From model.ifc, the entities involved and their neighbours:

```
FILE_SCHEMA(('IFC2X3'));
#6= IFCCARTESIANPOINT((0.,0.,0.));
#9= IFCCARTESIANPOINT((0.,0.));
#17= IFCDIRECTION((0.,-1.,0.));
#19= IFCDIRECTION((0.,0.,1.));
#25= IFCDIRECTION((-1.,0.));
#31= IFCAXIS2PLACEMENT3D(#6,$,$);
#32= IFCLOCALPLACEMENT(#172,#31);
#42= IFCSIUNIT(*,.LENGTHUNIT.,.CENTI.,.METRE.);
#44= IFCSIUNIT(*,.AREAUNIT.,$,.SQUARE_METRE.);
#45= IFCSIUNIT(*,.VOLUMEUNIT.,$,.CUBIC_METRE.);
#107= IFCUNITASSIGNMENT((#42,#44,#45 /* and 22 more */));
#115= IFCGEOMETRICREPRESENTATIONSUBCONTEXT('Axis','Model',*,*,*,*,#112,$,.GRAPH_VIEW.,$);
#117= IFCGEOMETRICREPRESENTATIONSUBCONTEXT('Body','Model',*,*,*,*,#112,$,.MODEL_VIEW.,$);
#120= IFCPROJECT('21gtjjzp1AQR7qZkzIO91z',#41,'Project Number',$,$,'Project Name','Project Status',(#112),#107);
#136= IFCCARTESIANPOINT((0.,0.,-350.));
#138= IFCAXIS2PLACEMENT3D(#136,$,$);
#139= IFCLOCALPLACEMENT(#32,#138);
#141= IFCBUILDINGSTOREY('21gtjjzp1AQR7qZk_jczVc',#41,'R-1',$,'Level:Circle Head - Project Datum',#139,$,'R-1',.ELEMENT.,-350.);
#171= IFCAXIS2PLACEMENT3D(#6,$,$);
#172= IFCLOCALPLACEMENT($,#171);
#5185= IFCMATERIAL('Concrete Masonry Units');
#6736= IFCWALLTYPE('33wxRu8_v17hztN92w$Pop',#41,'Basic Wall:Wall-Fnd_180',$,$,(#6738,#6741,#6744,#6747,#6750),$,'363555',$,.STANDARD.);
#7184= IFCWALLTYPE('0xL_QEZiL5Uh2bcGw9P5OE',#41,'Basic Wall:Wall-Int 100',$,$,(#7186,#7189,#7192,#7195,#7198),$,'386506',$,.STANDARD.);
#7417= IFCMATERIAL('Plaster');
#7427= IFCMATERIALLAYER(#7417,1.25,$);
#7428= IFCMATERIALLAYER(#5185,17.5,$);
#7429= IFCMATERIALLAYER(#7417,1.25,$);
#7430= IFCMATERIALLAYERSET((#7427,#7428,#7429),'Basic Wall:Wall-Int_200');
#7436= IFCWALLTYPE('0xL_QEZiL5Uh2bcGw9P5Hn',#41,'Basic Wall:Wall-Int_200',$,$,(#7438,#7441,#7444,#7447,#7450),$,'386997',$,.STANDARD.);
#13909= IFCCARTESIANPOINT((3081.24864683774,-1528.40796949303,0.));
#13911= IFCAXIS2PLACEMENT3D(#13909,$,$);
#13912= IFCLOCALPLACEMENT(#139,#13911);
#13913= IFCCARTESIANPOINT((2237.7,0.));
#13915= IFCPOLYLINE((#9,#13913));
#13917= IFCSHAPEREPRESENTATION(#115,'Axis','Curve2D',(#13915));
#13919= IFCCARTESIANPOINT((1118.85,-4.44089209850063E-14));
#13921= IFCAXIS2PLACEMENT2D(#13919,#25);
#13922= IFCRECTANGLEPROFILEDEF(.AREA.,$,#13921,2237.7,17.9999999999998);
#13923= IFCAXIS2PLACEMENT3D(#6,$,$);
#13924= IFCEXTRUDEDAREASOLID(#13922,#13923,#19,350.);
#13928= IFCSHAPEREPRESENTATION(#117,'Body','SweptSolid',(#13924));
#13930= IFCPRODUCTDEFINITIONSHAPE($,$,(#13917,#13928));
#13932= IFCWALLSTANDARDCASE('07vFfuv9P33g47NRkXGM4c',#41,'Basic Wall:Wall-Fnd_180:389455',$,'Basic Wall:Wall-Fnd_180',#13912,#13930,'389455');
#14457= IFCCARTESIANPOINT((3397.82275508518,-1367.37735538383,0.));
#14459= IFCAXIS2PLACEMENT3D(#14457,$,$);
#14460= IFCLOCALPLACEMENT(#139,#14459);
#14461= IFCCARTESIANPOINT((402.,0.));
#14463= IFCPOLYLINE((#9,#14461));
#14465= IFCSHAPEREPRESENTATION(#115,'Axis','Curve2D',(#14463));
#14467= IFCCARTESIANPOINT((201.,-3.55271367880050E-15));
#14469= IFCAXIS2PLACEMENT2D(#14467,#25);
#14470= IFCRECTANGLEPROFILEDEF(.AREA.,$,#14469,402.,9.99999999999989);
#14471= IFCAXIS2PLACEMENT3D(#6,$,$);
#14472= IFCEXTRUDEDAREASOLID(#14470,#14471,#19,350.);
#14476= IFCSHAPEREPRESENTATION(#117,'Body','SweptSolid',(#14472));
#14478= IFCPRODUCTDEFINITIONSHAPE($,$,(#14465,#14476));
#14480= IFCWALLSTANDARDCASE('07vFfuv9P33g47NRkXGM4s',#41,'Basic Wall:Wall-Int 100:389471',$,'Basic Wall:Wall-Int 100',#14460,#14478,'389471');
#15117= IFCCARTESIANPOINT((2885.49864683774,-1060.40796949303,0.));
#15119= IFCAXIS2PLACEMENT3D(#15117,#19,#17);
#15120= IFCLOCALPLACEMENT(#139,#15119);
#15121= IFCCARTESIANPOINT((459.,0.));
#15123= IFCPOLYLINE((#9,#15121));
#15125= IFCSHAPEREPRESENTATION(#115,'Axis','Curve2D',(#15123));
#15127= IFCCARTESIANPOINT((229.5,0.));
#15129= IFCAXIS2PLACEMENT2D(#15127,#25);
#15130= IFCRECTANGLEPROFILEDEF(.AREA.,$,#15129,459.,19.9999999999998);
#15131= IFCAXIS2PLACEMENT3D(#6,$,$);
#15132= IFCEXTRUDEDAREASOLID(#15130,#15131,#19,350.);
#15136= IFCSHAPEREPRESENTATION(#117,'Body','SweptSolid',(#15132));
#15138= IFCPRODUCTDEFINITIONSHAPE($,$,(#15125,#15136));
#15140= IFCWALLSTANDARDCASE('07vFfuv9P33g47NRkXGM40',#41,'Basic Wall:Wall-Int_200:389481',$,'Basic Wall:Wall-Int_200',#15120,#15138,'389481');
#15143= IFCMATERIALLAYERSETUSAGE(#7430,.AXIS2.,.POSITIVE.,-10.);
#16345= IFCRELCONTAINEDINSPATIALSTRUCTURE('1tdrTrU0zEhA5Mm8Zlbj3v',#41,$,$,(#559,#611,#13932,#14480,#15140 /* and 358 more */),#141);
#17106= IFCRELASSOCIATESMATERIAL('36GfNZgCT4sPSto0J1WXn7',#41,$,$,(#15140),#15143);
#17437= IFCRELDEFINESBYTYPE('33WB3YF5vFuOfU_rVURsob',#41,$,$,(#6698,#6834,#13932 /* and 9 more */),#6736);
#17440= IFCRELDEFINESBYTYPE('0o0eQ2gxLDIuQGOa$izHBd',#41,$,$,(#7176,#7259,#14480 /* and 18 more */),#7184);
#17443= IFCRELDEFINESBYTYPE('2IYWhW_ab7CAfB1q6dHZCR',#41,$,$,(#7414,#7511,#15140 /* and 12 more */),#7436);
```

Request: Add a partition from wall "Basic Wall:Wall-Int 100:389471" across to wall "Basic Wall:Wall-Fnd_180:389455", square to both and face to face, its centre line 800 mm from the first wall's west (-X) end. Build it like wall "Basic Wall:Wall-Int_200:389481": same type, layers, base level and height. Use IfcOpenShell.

```python
import numpy as np
import ifcopenshell
import ifcopenshell.api.geometry
import ifcopenshell.api.material
import ifcopenshell.api.pset
import ifcopenshell.api.root
import ifcopenshell.api.spatial
import ifcopenshell.api.type
import ifcopenshell.geom
import ifcopenshell.util.element
import ifcopenshell.util.placement
import ifcopenshell.util.representation
import ifcopenshell.util.shape
import ifcopenshell.util.unit

model = ifcopenshell.open("model.ifc")
unit_scale = ifcopenshell.util.unit.calculate_unit_scale(model)
settings = ifcopenshell.geom.settings()
settings.set("use-world-coords", True)

start_wall = model.by_id(14480)
end_wall = model.by_guid("07vFfuv9P33g47NRkXGM4c")
like = model.by_id(15140)
matrix = ifcopenshell.util.placement.get_local_placement(start_wall.ObjectPlacement)
matrix[:3, 3] *= unit_scale


def extent(element):
    """Bounding box in the first wall's axes, in metres."""
    shape = ifcopenshell.geom.create_shape(settings, element)
    points = (ifcopenshell.util.shape.get_vertices(shape.geometry) - matrix[:3, 3]) @ matrix[:3, :3]
    return points.min(axis=0), points.max(axis=0)


y_start = extent(start_wall)[0][1]
y_end = extent(end_wall)[1][1]
like_min, like_max = extent(like)
length, height = float(abs(y_end - y_start)), float(like_max[2] - like_min[2])
layer_set = ifcopenshell.util.element.get_material(like, should_skip_usage=True)
thickness = sum(layer.LayerThickness for layer in layer_set.MaterialLayers) * unit_scale

wall = ifcopenshell.api.root.create_entity(model, ifc_class="IfcWallStandardCase", name="New partition")
storey = ifcopenshell.util.element.get_container(like)
ifcopenshell.api.spatial.assign_container(model, products=[wall], relating_structure=storey)
ifcopenshell.api.type.assign_type(
    model, related_objects=[wall], relating_type=ifcopenshell.util.element.get_type(like), should_map_representations=False
)
rel = ifcopenshell.api.material.assign_material(
    model, products=[wall], type="IfcMaterialLayerSetUsage", material=layer_set
)
rel.RelatingMaterial.OffsetFromReferenceLine = -thickness / 2 / unit_scale
pset = ifcopenshell.api.pset.add_pset(model, product=wall, name="Pset_WallCommon")
ifcopenshell.api.pset.edit_pset(model, pset=pset, properties={"IsExternal": False, "LoadBearing": False})

# The axis runs down the middle of the wall.
axis = ifcopenshell.api.geometry.add_axis_representation(
    model, context=ifcopenshell.util.representation.get_context(model, "Model", "Axis"), axis=[(0.0, 0.0), (length, 0.0)]
)
body = ifcopenshell.api.geometry.add_wall_representation(
    model,
    context=ifcopenshell.util.representation.get_context(model, "Model", "Body", "MODEL_VIEW"),
    length=length,
    height=height,
    thickness=thickness,
    offset=-thickness / 2,
)
for representation in (axis, body):
    ifcopenshell.api.geometry.assign_representation(model, product=wall, representation=representation)

placement = matrix @ ifcopenshell.util.placement.rotation(-90, "Z")
placement[:, 3] = matrix @ np.array([extent(start_wall)[0][0] + 0.8, y_start, like_min[2], 1.0])
ifcopenshell.api.geometry.edit_object_placement(model, product=wall, matrix=placement)

print(f"partition {length:.3f} m long, {height:.3f} m high, {thickness:.3f} m thick")

model.write("model-out.ifc")
```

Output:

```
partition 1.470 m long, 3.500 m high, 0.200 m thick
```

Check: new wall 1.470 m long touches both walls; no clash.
